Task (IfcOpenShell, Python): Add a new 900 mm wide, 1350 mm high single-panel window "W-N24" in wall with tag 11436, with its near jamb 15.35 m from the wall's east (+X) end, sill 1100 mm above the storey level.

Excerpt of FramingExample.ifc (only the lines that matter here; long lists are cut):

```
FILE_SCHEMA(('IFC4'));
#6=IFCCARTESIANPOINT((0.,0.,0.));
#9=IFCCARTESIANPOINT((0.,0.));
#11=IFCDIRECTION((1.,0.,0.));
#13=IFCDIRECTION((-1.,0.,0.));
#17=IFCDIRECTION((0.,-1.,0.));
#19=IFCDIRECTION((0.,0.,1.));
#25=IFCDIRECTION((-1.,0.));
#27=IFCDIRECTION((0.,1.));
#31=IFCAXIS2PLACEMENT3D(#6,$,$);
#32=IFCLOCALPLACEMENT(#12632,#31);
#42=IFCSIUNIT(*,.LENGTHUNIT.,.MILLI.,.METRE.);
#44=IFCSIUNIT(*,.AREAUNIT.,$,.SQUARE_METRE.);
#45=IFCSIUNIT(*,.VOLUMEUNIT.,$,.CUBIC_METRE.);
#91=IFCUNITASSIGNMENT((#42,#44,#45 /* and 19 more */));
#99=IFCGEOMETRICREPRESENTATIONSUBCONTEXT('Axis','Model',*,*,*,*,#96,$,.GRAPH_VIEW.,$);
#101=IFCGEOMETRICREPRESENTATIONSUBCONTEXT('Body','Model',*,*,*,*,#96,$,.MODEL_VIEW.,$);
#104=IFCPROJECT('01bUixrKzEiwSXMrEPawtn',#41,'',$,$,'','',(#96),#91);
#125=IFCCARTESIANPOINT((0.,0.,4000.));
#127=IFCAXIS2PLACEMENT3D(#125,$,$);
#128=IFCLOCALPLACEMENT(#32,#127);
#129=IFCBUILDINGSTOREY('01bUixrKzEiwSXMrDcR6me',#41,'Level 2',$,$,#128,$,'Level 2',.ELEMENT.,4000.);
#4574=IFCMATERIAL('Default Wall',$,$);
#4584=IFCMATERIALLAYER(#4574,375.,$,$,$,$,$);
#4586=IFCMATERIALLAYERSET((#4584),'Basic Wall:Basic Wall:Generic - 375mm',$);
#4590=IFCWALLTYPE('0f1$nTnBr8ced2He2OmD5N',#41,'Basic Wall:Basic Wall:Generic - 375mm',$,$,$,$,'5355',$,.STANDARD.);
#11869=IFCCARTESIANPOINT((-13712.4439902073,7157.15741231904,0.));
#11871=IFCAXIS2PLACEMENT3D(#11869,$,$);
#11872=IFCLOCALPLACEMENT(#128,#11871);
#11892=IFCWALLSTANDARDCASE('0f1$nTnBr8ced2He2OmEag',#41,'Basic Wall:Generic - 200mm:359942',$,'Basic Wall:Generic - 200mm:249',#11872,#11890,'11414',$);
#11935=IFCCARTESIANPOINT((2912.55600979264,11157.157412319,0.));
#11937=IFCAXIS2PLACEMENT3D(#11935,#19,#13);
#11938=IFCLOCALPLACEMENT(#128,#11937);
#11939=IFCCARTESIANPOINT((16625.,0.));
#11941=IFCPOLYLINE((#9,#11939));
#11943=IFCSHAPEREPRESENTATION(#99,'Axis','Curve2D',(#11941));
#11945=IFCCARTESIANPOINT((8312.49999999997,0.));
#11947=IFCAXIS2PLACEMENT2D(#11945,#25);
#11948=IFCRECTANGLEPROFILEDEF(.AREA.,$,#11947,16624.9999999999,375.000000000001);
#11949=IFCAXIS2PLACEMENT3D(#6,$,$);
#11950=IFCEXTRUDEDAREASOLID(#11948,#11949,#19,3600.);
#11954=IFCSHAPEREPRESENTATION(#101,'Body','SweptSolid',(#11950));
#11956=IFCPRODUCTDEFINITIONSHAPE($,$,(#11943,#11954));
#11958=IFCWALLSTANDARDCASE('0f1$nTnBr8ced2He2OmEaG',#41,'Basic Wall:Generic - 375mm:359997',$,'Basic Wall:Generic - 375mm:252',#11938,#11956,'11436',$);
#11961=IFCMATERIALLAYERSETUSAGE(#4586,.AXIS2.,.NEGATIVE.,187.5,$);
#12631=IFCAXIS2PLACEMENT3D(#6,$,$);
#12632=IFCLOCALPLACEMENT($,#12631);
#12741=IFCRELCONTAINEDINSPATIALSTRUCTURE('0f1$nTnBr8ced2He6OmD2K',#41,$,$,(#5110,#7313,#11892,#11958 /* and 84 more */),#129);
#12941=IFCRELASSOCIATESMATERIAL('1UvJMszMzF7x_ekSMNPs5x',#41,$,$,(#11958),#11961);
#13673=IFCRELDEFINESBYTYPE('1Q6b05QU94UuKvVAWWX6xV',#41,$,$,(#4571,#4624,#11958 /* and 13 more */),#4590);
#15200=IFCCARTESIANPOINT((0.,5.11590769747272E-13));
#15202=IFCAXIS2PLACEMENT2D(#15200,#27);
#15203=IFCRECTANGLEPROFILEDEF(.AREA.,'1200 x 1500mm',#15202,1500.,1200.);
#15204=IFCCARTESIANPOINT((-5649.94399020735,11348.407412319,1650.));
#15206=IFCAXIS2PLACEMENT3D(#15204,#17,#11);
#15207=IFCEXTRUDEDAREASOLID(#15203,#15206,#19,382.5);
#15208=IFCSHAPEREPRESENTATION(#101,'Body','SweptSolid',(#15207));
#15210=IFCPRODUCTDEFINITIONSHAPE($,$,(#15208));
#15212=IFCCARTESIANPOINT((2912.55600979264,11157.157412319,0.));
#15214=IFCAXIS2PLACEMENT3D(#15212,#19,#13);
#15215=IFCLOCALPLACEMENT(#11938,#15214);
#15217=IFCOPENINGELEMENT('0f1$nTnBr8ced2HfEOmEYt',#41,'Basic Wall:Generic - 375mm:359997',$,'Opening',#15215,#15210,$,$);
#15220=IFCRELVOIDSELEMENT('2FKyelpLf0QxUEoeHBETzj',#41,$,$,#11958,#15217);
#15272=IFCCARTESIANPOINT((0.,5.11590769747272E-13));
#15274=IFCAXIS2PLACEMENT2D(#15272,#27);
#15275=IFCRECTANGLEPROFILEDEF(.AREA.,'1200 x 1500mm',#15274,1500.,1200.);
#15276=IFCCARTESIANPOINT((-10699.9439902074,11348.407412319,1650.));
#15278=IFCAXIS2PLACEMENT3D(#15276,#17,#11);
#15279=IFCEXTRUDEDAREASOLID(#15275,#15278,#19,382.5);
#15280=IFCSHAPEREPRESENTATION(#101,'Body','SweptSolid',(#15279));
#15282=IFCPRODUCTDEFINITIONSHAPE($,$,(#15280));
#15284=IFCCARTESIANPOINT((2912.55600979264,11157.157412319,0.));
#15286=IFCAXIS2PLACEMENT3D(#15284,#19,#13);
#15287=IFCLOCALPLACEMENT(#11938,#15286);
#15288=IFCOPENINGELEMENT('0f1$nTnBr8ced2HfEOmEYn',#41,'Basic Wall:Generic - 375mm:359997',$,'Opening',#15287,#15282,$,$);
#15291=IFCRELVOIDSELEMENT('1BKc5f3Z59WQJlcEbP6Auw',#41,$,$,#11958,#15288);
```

```python
import numpy as np
import ifcopenshell
import ifcopenshell.api.feature
import ifcopenshell.api.geometry
import ifcopenshell.api.root
import ifcopenshell.api.spatial
import ifcopenshell.geom
import ifcopenshell.util.element
import ifcopenshell.util.placement
import ifcopenshell.util.representation
import ifcopenshell.util.shape
import ifcopenshell.util.unit

model = ifcopenshell.open("FramingExample.ifc")
unit_scale = ifcopenshell.util.unit.calculate_unit_scale(model)
settings = ifcopenshell.geom.settings()


def volume(element):
    """Net volume in cubic metres, openings subtracted."""
    shape = ifcopenshell.geom.create_shape(settings, element)
    return ifcopenshell.util.shape.get_volume(shape.geometry)


wall = model.by_guid("0f1$nTnBr8ced2He2OmEaG")
storey = ifcopenshell.util.element.get_container(wall, ifc_class="IfcBuildingStorey")
context = ifcopenshell.util.representation.get_context(model, "Model", "Body", "MODEL_VIEW")
before = volume(wall)

width, height, from_end, sill = 0.9, 1.35, 15.35, 1.1  # metres

# The wall runs along its own X axis, and the end named is its -X end.
wall_shape = ifcopenshell.geom.create_shape(settings, wall)
x, y, z = ifcopenshell.util.shape.get_vertices(wall_shape.geometry).T
start = x.min() + from_end
face, thickness = float(y.min()), float(y.max() - y.min())
wall_matrix = ifcopenshell.util.placement.get_local_placement(wall.ObjectPlacement)
level = ifcopenshell.util.placement.get_local_placement(storey.ObjectPlacement)[2, 3]


def in_wall(x, y):
    """Placement at x, y metres in the wall's axes, at sill height."""
    matrix = wall_matrix.copy()
    matrix[:, 3] = wall_matrix @ np.array([x / unit_scale, y / unit_scale, 0.0, 1.0])
    matrix[2, 3] = level + sill / unit_scale
    return matrix


# Opening: a box that overshoots both wall faces by 50 mm.
opening = ifcopenshell.api.root.create_entity(model, ifc_class="IfcOpeningElement", predefined_type="OPENING")
box = ifcopenshell.api.geometry.add_wall_representation(
    model, context=context, length=width, height=height, thickness=thickness + 0.1
)
ifcopenshell.api.geometry.assign_representation(model, product=opening, representation=box)
ifcopenshell.api.geometry.edit_object_placement(model, product=opening, matrix=in_wall(start, face - 0.05), is_si=False)
ifcopenshell.api.feature.add_feature(model, feature=opening, element=wall)

window = ifcopenshell.api.root.create_entity(model, ifc_class="IfcWindow", name="W-N24", predefined_type="WINDOW")
window.OverallWidth, window.OverallHeight = width / unit_scale, height / unit_scale
window.PartitioningType = "SINGLE_PANEL"
body = ifcopenshell.api.geometry.add_window_representation(
    model,
    context=context,
    overall_width=window.OverallWidth,
    overall_height=window.OverallHeight,
    partition_type="SINGLE_PANEL",
)
ifcopenshell.api.geometry.assign_representation(model, product=window, representation=body)
ifcopenshell.api.spatial.assign_container(model, products=[window], relating_structure=storey)
ifcopenshell.api.feature.add_filling(model, opening=opening, element=window)

# Centre the window in the wall's thickness.
ifcopenshell.api.geometry.edit_object_placement(model, product=window, matrix=in_wall(start, face), is_si=False)
window_shape = ifcopenshell.geom.create_shape(settings, window)
depth = ifcopenshell.util.shape.get_vertices(window_shape.geometry)[:, 1]
offset = face + thickness / 2 - (depth.min() + depth.max()) / 2
ifcopenshell.api.geometry.edit_object_placement(model, product=window, matrix=in_wall(start, offset), is_si=False)

after = volume(wall)

print(f"wall volume {before:.3f} -> {after:.3f} m3")

model.write("FramingExample_v2.ifc")
```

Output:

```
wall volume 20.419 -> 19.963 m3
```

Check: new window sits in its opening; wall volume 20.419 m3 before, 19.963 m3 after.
